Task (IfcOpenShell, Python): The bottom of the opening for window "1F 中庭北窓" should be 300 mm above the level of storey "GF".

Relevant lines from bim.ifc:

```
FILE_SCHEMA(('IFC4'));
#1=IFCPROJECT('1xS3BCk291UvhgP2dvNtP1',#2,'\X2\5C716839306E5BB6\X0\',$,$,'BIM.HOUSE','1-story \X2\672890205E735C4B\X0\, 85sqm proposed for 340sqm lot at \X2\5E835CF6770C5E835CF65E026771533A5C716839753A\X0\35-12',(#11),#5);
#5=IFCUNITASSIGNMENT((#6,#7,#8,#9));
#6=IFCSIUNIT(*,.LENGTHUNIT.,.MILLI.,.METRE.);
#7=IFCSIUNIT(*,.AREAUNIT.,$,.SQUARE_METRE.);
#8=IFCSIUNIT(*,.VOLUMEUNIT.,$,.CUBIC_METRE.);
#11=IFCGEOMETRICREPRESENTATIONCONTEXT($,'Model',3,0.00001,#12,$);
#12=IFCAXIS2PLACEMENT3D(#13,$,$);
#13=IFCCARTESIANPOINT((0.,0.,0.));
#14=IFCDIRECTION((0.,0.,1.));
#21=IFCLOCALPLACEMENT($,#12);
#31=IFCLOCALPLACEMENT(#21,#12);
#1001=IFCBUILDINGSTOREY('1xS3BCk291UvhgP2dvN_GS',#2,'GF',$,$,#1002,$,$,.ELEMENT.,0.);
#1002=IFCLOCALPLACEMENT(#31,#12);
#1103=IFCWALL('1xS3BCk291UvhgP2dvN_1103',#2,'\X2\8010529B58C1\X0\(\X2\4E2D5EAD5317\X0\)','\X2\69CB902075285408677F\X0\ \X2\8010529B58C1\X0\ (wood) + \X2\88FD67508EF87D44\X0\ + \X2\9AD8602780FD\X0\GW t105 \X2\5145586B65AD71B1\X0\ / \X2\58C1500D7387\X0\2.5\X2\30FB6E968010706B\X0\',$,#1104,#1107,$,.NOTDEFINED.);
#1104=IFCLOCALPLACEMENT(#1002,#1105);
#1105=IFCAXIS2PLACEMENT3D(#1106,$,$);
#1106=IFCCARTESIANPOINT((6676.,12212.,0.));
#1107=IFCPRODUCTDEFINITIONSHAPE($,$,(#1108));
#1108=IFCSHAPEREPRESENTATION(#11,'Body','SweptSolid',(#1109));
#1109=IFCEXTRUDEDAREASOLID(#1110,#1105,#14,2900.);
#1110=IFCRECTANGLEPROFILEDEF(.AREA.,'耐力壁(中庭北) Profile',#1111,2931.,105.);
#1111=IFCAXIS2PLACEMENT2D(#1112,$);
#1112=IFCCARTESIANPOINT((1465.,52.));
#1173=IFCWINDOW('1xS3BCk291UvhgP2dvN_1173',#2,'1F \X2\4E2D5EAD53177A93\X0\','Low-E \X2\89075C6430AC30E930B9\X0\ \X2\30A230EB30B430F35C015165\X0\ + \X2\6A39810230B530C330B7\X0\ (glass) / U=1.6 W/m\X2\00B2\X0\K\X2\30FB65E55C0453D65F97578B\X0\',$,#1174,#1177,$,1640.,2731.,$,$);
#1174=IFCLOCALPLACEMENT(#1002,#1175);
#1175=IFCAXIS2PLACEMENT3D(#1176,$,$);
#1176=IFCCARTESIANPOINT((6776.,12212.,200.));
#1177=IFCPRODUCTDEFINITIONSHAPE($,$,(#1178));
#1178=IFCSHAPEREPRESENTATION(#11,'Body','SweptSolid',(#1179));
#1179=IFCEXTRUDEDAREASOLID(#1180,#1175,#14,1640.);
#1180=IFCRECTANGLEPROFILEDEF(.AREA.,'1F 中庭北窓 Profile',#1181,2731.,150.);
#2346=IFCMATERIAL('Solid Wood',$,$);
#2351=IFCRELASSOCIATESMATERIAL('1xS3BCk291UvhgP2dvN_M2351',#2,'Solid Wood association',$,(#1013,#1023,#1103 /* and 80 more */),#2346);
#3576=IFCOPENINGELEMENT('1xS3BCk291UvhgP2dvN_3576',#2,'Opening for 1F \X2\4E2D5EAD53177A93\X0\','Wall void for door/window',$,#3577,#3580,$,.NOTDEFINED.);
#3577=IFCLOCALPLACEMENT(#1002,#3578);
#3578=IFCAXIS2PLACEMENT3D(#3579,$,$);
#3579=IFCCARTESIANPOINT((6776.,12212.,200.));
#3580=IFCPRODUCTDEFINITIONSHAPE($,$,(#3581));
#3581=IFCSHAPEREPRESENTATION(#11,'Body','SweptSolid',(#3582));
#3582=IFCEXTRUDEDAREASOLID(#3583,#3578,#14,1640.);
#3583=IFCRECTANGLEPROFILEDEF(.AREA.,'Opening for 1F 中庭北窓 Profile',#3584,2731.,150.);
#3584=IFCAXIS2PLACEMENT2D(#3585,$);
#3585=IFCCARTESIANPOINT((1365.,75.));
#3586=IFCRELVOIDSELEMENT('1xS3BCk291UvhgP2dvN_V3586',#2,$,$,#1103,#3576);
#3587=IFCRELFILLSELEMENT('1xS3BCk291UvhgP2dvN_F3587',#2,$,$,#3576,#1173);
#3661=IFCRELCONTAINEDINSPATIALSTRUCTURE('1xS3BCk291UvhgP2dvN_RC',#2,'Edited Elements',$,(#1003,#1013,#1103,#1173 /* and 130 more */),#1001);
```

```python
import numpy as np
import ifcopenshell
import ifcopenshell.api.geometry
import ifcopenshell.geom
import ifcopenshell.util.element
import ifcopenshell.util.placement
import ifcopenshell.util.shape
import ifcopenshell.util.unit

model = ifcopenshell.open("bim.ifc")
unit_scale = ifcopenshell.util.unit.calculate_unit_scale(model)

window = model.by_guid("1xS3BCk291UvhgP2dvN_1173")
opening = window.FillsVoids[0].RelatingOpeningElement
storey = ifcopenshell.util.element.get_container(window, ifc_class="IfcBuildingStorey")
level = ifcopenshell.util.placement.get_local_placement(storey.ObjectPlacement)[2, 3]

# The opening's origin need not be at the sill, so measure its lowest point.
shape = ifcopenshell.geom.create_shape(ifcopenshell.geom.settings(), opening)
bottom = ifcopenshell.util.shape.get_shape_bottom_elevation(shape, shape.geometry) / unit_scale
dz = level + 300.0 - bottom

shift = np.array([0.0, 0.0, dz])
# The window is not placed relative to its opening, so move both.
for product in (opening, window):
    matrix = ifcopenshell.util.placement.get_local_placement(product.ObjectPlacement)
    matrix[:3, 3] += shift
    ifcopenshell.api.geometry.edit_object_placement(model, product=product, matrix=matrix, is_si=False)

print(f"moved by {dz * unit_scale:+.3f} m")

model.write("bim_rev.ifc")
```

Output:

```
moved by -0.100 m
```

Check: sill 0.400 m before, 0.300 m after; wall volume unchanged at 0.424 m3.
